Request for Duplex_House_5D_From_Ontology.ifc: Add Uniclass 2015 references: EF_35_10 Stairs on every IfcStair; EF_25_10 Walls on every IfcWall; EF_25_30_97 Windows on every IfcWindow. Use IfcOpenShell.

First a look at what the model holds.

```python
import ifcopenshell

model = ifcopenshell.open("Duplex_House_5D_From_Ontology.ifc")
print(model.schema)
print("classifications:", [c.Name for c in model.by_type("IfcClassification")])
for ifc_class in ("IfcDoor", "IfcRoof", "IfcStair", "IfcWall", "IfcWindow"):
    print(ifc_class, len(model.by_type(ifc_class)))
```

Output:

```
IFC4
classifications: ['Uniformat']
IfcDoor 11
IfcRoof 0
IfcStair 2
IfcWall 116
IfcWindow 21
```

```python
import ifcopenshell
import ifcopenshell.api.classification

model = ifcopenshell.open("Duplex_House_5D_From_Ontology.ifc")

system = ifcopenshell.api.classification.add_classification(model, classification="Uniclass 2015")

codes = {
    "IfcStair": ("EF_35_10", "Stairs"),
    "IfcWall": ("EF_25_10", "Walls"),
    "IfcWindow": ("EF_25_30_97", "Windows"),
}
for ifc_class, (code, name) in codes.items():
    products = model.by_type(ifc_class)
    ifcopenshell.api.classification.add_reference(
        model, products=products, classification=system, identification=code, name=name
    )
    print(code, len(products))

model.write("Duplex_House_5D_From_Ontology_v2.ifc")
```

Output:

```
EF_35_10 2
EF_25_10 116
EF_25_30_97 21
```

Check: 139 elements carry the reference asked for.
